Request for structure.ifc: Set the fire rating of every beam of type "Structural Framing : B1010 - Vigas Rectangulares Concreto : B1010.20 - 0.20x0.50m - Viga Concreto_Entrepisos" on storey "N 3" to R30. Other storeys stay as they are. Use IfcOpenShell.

First a look at what the model holds.

```python
import ifcopenshell
import ifcopenshell.util.element

model = ifcopenshell.open("structure.ifc")
print(model.schema)
storey = next(s for s in model.by_type("IfcBuildingStorey") if s.Name == "N 3")
beams = [e for e in ifcopenshell.util.element.get_decomposition(storey) if e.is_a("IfcBeam")]
seen = {}
for e in beams:
    element_type = ifcopenshell.util.element.get_type(e)
    key = (element_type.Name if element_type != e and element_type else None, ifcopenshell.util.element.get_pset(e, "Pset_BeamCommon", "FireRating"))
    seen[key] = seen.get(key, 0) + 1
for (name, value), count in sorted(seen.items(), key=str):
    print(count, "x", name, "|", value)
```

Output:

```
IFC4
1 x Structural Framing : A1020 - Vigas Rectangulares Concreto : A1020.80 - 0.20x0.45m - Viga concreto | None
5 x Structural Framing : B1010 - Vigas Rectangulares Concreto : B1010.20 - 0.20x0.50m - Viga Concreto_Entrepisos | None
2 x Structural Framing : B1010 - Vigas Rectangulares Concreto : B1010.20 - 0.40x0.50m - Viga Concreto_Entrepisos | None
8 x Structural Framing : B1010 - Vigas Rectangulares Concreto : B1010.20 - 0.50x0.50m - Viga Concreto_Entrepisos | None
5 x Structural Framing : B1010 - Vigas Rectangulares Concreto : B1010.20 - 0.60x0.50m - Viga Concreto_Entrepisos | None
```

```python
import ifcopenshell
import ifcopenshell.api.pset
import ifcopenshell.util.element

model = ifcopenshell.open("structure.ifc")

storey = next(s for s in model.by_type("IfcBuildingStorey") if s.Name == "N 3")
beams = [e for e in ifcopenshell.util.element.get_decomposition(storey) if e.is_a("IfcBeam")]

count = 0
for e in beams:
    element_type = ifcopenshell.util.element.get_type(e)
    if element_type in (None, e) or element_type.Name != "Structural Framing : B1010 - Vigas Rectangulares Concreto : B1010.20 - 0.20x0.50m - Viga Concreto_Entrepisos":
        continue
    # add_pset returns the element's existing set when there is one.
    pset = ifcopenshell.api.pset.add_pset(model, product=e, name="Pset_BeamCommon")
    ifcopenshell.api.pset.edit_pset(model, pset=pset, properties={"FireRating": "R30"})
    count += 1

print(count, "beams updated")

model.write("structure_rev.ifc")
```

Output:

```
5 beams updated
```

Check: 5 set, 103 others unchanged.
